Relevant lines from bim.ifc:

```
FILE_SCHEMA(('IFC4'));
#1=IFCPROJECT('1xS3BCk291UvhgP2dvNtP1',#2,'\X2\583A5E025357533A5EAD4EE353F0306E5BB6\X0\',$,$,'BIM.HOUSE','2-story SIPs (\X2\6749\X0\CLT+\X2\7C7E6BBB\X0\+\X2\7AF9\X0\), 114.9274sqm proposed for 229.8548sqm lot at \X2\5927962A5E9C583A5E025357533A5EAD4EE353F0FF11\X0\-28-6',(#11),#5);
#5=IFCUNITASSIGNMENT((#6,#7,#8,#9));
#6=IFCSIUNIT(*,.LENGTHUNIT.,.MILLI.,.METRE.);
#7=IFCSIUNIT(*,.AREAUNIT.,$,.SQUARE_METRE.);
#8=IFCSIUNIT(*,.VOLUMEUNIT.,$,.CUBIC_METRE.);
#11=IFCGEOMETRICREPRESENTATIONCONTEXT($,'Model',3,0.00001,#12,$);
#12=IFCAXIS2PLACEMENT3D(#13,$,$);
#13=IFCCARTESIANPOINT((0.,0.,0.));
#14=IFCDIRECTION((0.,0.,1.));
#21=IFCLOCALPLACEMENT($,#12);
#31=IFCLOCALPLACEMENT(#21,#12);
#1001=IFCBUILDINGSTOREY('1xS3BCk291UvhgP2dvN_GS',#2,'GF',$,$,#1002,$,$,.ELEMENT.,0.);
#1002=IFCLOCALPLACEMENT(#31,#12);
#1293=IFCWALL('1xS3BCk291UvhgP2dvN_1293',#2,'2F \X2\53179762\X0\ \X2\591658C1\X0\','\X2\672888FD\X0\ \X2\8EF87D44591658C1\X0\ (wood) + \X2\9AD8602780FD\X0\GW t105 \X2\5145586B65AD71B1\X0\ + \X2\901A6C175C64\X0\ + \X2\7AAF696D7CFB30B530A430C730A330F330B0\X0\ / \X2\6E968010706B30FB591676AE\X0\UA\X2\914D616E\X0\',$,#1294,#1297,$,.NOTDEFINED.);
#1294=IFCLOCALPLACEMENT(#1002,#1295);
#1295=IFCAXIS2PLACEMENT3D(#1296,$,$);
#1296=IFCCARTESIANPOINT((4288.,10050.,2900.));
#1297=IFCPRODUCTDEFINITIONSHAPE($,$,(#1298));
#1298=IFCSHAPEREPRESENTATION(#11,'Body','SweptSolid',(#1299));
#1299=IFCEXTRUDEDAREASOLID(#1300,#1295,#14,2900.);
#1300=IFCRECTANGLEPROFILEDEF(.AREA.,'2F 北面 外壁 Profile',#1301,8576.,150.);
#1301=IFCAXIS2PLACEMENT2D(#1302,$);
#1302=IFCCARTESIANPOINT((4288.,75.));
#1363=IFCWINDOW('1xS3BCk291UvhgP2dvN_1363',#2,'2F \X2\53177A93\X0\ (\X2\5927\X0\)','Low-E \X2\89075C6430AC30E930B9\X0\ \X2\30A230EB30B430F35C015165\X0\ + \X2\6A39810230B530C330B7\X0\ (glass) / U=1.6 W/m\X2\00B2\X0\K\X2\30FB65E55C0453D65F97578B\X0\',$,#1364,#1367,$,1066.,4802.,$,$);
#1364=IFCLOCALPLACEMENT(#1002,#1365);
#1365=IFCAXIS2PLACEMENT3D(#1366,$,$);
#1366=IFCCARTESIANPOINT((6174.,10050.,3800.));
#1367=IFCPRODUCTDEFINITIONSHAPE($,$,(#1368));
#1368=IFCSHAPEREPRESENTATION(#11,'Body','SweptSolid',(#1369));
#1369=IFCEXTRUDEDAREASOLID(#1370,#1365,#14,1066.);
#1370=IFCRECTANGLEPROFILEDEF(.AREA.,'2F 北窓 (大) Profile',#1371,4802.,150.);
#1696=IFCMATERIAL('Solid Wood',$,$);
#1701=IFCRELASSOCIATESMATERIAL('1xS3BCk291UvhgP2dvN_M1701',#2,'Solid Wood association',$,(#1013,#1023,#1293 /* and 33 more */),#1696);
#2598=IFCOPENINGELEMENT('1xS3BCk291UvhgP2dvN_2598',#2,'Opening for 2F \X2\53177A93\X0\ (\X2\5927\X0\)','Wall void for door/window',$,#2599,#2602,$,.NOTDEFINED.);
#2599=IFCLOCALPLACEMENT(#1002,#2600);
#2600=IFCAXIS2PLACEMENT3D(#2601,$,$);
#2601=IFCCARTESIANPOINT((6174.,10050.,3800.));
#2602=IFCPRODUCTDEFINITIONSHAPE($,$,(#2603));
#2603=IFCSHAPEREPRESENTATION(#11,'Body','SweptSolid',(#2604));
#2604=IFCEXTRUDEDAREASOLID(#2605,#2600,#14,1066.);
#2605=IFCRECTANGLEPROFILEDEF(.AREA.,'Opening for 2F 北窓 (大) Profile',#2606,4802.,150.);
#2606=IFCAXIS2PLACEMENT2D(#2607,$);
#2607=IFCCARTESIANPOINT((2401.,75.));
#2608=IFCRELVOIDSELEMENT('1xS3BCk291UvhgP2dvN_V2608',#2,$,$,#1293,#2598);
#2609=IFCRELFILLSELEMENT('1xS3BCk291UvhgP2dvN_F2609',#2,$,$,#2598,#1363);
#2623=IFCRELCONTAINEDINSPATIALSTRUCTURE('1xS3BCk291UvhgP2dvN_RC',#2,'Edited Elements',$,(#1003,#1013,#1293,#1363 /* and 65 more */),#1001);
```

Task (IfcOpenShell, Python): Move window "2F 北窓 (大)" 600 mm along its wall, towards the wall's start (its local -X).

```python
import ifcopenshell
import ifcopenshell.api.geometry
import ifcopenshell.util.placement
import ifcopenshell.util.unit

model = ifcopenshell.open("bim.ifc")
unit_scale = ifcopenshell.util.unit.calculate_unit_scale(model)

window = model.by_guid("1xS3BCk291UvhgP2dvN_1363")
opening = window.FillsVoids[0].RelatingOpeningElement
wall = opening.VoidsElements[0].RelatingBuildingElement

wall_matrix = ifcopenshell.util.placement.get_local_placement(wall.ObjectPlacement)
shift = wall_matrix[:3, 0] * -0.6 / unit_scale
before = ifcopenshell.util.placement.get_local_placement(window.ObjectPlacement)[:3, 3].copy()

# The window is not placed relative to its opening, so move both.
for product in (opening, window):
    matrix = ifcopenshell.util.placement.get_local_placement(product.ObjectPlacement)
    matrix[:3, 3] += shift
    ifcopenshell.api.geometry.edit_object_placement(model, product=product, matrix=matrix, is_si=False)

after = ifcopenshell.util.placement.get_local_placement(window.ObjectPlacement)[:3, 3]
print("window moved by", (after - before).round(3) + 0.0)

model.write("bim_rev.ifc")
```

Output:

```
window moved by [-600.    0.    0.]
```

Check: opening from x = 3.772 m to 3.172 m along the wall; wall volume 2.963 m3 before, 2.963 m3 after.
